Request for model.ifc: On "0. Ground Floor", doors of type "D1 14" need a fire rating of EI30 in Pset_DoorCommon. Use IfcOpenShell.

First a look at what the model holds.

```python
import ifcopenshell
import ifcopenshell.util.element

model = ifcopenshell.open("model.ifc")
print(model.schema)
storey = next(s for s in model.by_type("IfcBuildingStorey") if s.Name == "0. Ground Floor")
doors = [e for e in ifcopenshell.util.element.get_decomposition(storey) if e.is_a("IfcDoor")]
seen = {}
for e in doors:
    element_type = ifcopenshell.util.element.get_type(e)
    key = (element_type.Name if element_type != e and element_type else None, ifcopenshell.util.element.get_pset(e, "Pset_DoorCommon", "FireRating"))
    seen[key] = seen.get(key, 0) + 1
for (name, value), count in sorted(seen.items(), key=str):
    print(count, "x", name, "|", value)
```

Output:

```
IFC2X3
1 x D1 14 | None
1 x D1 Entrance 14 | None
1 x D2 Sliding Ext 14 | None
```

```python
import ifcopenshell
import ifcopenshell.api.pset
import ifcopenshell.util.element

model = ifcopenshell.open("model.ifc")

storey = next(s for s in model.by_type("IfcBuildingStorey") if s.Name == "0. Ground Floor")
doors = [e for e in ifcopenshell.util.element.get_decomposition(storey) if e.is_a("IfcDoor")]

count = 0
for e in doors:
    element_type = ifcopenshell.util.element.get_type(e)
    if element_type in (None, e) or element_type.Name != "D1 14":
        continue
    # add_pset returns the element's existing set when there is one.
    pset = ifcopenshell.api.pset.add_pset(model, product=e, name="Pset_DoorCommon")
    ifcopenshell.api.pset.edit_pset(model, pset=pset, properties={"FireRating": "EI30"})
    count += 1

print(count, "doors updated")

model.write("model_updated.ifc")
```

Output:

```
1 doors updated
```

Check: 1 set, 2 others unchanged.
